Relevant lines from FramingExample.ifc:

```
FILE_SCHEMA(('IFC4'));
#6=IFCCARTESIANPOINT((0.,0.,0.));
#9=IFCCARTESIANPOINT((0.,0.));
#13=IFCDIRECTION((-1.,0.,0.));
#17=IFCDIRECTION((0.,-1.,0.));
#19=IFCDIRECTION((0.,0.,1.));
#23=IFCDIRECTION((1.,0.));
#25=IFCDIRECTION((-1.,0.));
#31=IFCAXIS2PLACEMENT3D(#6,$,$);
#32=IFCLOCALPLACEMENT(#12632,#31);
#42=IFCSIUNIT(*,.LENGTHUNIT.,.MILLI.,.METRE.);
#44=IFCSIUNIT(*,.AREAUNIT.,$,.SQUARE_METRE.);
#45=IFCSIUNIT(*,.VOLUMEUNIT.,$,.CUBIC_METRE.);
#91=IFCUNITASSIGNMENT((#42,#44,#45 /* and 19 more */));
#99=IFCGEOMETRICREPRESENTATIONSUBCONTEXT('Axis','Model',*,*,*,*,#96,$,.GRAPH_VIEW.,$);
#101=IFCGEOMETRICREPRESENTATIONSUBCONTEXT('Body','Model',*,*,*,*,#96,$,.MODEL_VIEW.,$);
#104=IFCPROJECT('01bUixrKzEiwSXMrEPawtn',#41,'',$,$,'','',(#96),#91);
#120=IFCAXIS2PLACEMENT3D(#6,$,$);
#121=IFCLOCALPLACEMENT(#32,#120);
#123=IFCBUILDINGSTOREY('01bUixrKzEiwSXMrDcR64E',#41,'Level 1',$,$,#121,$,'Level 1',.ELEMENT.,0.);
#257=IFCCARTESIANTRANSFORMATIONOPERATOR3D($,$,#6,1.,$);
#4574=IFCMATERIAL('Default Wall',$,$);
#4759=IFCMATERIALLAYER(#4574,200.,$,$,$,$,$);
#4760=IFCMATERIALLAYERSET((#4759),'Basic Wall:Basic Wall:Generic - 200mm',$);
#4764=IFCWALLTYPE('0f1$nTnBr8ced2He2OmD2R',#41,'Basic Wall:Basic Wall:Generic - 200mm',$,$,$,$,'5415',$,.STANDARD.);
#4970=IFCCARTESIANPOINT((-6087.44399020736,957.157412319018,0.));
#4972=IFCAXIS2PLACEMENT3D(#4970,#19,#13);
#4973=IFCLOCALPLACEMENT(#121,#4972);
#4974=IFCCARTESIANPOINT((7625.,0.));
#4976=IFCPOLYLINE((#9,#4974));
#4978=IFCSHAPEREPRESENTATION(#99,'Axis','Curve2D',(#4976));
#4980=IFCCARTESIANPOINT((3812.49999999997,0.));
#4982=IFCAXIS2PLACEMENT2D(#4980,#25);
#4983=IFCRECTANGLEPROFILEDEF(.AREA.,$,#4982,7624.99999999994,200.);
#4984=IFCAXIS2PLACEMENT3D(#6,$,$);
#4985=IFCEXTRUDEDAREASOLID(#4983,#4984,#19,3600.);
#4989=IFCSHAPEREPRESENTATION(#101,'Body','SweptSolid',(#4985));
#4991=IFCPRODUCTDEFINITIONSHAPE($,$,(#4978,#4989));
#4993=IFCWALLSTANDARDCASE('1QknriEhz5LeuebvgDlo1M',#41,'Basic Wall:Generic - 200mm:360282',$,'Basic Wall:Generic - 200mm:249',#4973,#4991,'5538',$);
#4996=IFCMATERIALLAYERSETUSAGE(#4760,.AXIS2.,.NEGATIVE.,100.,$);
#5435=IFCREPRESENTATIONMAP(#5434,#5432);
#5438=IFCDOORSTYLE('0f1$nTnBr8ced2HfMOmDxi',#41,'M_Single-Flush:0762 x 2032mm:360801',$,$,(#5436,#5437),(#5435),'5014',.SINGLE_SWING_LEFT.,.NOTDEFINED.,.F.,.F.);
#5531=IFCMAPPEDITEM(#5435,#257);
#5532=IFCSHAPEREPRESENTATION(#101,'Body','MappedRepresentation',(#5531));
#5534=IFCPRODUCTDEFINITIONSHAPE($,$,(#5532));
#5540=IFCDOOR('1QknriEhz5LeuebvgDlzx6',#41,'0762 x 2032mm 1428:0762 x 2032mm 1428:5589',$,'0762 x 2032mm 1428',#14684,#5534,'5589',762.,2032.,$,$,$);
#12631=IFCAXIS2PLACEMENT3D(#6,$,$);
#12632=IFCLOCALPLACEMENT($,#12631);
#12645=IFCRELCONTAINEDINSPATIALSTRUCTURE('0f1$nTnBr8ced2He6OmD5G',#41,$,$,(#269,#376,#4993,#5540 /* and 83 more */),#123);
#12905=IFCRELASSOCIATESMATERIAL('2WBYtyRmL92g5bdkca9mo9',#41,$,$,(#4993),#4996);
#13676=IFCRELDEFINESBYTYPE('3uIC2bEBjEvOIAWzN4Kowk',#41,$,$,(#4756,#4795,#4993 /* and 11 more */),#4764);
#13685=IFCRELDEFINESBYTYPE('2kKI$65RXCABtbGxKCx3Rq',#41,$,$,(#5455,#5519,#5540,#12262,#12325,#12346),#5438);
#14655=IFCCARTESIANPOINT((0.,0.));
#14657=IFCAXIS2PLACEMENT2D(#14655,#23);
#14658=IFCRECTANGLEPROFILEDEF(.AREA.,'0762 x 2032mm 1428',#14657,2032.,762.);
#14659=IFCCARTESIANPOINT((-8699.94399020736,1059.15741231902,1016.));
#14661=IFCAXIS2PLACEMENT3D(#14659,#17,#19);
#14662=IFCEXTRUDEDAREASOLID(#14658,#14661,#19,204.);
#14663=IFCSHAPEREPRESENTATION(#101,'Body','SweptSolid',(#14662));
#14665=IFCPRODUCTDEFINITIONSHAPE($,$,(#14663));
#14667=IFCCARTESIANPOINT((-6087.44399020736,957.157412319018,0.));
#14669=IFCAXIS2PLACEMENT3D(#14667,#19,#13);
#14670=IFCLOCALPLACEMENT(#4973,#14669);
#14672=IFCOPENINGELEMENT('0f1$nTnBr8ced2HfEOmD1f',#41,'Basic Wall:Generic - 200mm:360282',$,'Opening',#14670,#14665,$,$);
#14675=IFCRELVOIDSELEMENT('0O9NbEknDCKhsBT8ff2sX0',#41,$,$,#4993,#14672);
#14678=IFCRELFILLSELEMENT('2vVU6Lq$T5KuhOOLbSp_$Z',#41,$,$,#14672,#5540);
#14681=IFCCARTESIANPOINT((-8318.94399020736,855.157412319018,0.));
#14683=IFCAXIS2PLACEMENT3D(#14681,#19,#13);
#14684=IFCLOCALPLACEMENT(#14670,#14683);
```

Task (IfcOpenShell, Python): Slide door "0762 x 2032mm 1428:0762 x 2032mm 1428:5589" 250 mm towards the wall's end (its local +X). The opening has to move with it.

```python
import ifcopenshell
import ifcopenshell.api.geometry
import ifcopenshell.util.placement

model = ifcopenshell.open("FramingExample.ifc")

door = model.by_id(5540)
opening = door.FillsVoids[0].RelatingOpeningElement
wall = opening.VoidsElements[0].RelatingBuildingElement

wall_matrix = ifcopenshell.util.placement.get_local_placement(wall.ObjectPlacement)
shift = wall_matrix[:3, 0] * 250.0
before = ifcopenshell.util.placement.get_local_placement(door.ObjectPlacement)[:3, 3].copy()

# The door is placed relative to its opening, so it follows when the opening moves.
matrix = ifcopenshell.util.placement.get_local_placement(opening.ObjectPlacement)
matrix[:3, 3] += shift
ifcopenshell.api.geometry.edit_object_placement(
    model, product=opening, matrix=matrix, is_si=False, should_transform_children=True
)

after = ifcopenshell.util.placement.get_local_placement(door.ObjectPlacement)[:3, 3]
print("door moved by", (after - before).round(3) + 0.0)

model.write("FramingExample_v2.ifc")
```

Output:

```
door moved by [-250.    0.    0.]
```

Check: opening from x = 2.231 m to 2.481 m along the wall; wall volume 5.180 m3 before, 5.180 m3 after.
